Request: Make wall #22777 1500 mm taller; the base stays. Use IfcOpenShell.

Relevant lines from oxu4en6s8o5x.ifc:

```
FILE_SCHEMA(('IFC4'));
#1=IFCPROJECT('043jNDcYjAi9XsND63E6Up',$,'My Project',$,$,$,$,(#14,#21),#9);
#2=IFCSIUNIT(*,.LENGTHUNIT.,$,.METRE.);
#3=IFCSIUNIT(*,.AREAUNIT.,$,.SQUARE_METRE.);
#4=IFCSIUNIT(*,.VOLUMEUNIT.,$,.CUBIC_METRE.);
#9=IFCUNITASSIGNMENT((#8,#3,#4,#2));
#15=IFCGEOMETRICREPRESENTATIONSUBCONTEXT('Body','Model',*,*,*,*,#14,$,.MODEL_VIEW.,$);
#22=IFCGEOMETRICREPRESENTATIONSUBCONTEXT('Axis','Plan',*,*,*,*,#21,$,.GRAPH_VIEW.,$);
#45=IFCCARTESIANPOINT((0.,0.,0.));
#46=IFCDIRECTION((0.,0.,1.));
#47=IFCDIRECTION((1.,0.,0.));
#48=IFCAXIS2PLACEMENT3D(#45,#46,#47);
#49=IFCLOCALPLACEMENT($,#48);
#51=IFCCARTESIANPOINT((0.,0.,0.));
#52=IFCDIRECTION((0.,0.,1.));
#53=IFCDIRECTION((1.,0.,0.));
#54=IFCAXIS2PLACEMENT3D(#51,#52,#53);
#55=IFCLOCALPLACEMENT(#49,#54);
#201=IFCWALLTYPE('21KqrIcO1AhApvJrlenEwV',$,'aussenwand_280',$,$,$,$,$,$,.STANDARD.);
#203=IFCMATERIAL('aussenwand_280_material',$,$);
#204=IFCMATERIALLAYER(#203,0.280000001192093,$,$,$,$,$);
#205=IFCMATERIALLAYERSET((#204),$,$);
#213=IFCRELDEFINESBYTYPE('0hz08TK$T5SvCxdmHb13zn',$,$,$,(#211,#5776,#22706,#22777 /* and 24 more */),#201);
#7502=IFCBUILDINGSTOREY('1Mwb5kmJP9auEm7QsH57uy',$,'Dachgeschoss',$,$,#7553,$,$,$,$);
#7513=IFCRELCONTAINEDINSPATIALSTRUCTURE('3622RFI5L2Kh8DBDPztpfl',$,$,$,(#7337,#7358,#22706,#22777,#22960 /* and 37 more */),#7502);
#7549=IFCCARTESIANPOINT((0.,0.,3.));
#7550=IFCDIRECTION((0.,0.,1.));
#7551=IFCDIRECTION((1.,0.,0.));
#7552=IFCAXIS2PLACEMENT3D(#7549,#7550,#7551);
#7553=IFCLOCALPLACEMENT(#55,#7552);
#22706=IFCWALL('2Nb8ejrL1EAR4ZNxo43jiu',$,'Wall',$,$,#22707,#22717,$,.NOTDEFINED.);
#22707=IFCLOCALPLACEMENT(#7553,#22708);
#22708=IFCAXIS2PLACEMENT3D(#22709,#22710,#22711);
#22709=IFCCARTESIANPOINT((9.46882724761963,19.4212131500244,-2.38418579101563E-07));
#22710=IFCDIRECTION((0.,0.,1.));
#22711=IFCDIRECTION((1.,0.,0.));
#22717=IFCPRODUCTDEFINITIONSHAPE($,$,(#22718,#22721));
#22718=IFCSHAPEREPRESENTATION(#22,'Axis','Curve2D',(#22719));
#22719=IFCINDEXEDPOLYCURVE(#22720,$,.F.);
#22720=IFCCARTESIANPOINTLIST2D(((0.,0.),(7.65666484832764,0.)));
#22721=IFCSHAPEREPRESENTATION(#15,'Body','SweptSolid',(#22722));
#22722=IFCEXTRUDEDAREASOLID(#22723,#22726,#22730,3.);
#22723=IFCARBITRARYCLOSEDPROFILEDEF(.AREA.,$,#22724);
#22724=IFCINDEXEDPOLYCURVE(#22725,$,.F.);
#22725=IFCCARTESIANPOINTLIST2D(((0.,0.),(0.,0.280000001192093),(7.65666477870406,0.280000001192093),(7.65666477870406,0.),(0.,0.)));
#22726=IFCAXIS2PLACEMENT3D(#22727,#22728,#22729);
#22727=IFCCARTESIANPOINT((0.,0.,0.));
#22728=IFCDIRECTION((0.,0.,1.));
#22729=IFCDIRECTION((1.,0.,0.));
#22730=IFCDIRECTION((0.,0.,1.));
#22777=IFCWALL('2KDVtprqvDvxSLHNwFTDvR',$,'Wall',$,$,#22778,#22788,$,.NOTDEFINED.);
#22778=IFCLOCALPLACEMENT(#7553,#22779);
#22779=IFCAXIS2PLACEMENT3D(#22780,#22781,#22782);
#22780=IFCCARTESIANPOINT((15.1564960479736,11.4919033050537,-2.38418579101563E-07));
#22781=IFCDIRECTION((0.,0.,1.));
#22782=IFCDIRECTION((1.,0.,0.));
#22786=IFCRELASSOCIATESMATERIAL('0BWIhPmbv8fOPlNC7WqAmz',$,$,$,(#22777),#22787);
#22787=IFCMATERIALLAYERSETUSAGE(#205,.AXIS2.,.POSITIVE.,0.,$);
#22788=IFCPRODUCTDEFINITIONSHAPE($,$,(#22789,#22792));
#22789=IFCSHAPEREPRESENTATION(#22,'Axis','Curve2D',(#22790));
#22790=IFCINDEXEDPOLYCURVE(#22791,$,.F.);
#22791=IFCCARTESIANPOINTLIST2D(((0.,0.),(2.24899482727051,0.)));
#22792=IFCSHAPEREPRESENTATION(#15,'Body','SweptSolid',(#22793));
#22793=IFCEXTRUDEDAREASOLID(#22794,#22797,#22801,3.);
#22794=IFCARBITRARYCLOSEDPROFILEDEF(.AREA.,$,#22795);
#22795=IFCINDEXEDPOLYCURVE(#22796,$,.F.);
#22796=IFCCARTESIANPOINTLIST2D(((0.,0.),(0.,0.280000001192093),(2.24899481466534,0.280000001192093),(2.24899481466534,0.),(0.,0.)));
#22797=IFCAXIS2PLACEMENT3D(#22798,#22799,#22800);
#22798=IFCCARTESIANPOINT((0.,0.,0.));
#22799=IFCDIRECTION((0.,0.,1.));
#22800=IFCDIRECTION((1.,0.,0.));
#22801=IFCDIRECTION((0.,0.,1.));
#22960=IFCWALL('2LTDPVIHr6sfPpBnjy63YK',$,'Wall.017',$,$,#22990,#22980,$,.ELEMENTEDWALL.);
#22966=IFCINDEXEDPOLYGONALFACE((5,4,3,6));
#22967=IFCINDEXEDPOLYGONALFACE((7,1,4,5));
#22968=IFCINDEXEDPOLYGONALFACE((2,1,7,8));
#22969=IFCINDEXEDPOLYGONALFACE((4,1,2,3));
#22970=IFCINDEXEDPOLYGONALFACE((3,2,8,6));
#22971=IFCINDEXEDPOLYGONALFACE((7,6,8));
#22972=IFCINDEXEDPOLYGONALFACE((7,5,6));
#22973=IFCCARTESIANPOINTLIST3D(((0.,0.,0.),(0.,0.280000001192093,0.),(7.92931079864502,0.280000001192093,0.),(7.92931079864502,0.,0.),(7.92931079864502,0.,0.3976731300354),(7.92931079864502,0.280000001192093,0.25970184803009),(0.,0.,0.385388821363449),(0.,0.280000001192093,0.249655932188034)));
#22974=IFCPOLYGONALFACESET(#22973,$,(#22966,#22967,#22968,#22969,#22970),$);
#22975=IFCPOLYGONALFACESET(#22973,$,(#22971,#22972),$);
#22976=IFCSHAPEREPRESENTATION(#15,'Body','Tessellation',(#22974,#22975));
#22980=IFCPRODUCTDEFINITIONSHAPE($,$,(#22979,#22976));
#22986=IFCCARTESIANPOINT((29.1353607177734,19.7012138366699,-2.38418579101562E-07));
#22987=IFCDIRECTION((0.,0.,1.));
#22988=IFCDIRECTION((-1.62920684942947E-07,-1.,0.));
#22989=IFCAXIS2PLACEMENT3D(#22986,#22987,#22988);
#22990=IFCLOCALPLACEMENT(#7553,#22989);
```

```python
import ifcopenshell
import ifcopenshell.geom
import ifcopenshell.util.representation
import ifcopenshell.util.shape
import ifcopenshell.util.unit

model = ifcopenshell.open("oxu4en6s8o5x.ifc")
unit_scale = ifcopenshell.util.unit.calculate_unit_scale(model)
settings = ifcopenshell.geom.settings()


def volume(element):
    """Net volume in cubic metres, openings subtracted."""
    shape = ifcopenshell.geom.create_shape(settings, element)
    return ifcopenshell.util.shape.get_volume(shape.geometry)


wall = model.by_guid("2KDVtprqvDvxSLHNwFTDvR")
before = volume(wall)

body = ifcopenshell.util.representation.get_representation(wall, "Model", "Body")
solid = body.Items[0]
old_height = solid.Depth
solid.Depth += 1.5 / unit_scale
after = volume(wall)

print(f"height {old_height:g} -> {solid.Depth:g}, volume {before:.3f} -> {after:.3f} m3")

model.write("oxu4en6s8o5x_v2.ifc")
```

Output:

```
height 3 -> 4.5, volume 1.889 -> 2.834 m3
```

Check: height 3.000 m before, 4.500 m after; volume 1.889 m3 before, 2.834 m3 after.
